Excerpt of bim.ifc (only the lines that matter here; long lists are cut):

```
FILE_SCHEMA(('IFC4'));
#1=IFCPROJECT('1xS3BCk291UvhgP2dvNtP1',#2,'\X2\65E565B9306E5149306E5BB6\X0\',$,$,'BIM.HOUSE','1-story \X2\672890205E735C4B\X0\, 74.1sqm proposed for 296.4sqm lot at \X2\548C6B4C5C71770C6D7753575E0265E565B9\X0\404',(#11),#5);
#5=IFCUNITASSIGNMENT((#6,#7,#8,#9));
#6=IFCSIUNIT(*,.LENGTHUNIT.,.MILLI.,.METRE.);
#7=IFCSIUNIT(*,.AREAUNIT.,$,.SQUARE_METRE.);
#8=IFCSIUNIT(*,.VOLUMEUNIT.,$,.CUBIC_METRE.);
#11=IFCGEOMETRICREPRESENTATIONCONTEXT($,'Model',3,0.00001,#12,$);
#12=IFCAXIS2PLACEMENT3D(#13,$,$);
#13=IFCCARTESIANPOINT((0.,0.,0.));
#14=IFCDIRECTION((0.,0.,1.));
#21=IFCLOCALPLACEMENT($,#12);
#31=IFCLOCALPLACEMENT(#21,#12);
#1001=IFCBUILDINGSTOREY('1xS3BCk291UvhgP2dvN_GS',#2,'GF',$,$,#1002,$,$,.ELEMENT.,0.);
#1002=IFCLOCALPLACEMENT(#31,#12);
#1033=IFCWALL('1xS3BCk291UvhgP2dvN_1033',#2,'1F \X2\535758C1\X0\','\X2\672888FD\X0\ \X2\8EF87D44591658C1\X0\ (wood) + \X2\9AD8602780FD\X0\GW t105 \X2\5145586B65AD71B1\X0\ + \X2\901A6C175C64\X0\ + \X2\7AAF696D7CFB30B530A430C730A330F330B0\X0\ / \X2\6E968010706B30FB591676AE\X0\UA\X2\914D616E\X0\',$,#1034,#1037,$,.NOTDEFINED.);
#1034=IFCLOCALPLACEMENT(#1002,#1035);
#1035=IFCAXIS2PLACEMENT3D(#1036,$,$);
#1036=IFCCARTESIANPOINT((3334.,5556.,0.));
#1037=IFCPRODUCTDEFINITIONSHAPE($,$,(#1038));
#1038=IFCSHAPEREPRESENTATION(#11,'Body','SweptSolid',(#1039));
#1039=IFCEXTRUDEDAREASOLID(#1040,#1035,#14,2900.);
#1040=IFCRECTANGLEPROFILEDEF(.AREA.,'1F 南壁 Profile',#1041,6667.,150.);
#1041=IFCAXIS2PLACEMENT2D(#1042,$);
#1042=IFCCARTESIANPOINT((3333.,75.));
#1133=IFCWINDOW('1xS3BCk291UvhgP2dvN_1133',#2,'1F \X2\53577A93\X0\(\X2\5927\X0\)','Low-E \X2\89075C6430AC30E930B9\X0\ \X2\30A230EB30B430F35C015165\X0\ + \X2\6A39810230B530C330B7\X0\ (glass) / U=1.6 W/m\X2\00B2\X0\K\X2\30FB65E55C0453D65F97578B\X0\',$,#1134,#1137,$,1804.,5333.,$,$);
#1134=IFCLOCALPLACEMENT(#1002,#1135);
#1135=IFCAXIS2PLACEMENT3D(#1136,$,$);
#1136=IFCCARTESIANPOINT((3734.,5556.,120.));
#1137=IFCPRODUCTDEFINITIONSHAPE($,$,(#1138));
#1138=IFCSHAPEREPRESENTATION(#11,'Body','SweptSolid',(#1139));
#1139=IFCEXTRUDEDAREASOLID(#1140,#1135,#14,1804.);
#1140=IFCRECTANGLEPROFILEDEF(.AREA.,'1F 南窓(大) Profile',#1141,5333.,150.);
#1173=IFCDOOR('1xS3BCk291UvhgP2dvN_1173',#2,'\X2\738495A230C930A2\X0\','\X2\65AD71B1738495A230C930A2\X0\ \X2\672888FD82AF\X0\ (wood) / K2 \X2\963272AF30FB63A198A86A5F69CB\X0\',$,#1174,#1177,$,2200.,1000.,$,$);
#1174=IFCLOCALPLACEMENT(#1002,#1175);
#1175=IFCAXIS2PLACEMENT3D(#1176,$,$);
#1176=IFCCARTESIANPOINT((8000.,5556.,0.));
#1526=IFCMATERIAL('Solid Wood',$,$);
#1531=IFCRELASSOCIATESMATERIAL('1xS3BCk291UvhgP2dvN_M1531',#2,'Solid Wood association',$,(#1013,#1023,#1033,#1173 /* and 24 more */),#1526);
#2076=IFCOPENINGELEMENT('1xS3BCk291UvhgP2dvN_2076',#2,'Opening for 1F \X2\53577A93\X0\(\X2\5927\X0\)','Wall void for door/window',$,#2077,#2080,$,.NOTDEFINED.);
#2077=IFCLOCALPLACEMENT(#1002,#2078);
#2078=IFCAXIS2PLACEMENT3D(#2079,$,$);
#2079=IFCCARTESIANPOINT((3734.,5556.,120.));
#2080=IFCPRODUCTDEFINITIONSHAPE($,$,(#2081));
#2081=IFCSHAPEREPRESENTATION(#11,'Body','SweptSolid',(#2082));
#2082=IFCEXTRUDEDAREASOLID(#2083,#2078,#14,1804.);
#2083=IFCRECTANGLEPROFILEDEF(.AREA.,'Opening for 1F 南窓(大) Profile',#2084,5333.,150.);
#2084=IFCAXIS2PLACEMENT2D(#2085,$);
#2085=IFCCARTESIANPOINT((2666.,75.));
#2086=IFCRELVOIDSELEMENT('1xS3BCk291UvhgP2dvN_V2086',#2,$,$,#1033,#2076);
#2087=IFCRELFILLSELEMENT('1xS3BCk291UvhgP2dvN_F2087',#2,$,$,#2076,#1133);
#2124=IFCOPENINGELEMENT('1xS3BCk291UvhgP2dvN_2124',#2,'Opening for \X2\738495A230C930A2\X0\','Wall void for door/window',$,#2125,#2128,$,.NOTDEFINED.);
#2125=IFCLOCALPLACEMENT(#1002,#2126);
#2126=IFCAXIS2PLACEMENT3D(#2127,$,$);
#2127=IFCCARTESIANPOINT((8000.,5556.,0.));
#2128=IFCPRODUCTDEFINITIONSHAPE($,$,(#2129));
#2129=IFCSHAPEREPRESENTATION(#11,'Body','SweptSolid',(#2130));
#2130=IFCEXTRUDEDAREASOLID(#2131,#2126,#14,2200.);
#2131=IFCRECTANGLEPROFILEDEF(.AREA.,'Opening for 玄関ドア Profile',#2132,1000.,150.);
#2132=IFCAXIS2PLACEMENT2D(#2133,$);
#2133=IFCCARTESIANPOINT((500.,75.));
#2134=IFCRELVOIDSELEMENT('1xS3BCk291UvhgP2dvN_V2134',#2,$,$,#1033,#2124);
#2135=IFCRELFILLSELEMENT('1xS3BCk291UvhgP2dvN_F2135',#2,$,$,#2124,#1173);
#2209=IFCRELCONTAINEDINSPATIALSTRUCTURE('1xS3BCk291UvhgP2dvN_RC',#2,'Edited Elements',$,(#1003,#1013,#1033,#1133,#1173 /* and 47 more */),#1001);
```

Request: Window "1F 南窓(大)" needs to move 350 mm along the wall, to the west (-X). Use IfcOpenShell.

```python
import ifcopenshell
import ifcopenshell.api.geometry
import ifcopenshell.util.placement

model = ifcopenshell.open("bim.ifc")

window = model.by_guid("1xS3BCk291UvhgP2dvN_1133")
opening = window.FillsVoids[0].RelatingOpeningElement
wall = opening.VoidsElements[0].RelatingBuildingElement

wall_matrix = ifcopenshell.util.placement.get_local_placement(wall.ObjectPlacement)
shift = wall_matrix[:3, 0] * -350.0
before = ifcopenshell.util.placement.get_local_placement(window.ObjectPlacement)[:3, 3].copy()

# The window is not placed relative to its opening, so move both.
for product in (opening, window):
    matrix = ifcopenshell.util.placement.get_local_placement(product.ObjectPlacement)
    matrix[:3, 3] += shift
    ifcopenshell.api.geometry.edit_object_placement(model, product=product, matrix=matrix, is_si=False)

after = ifcopenshell.util.placement.get_local_placement(window.ObjectPlacement)[:3, 3]
print("window moved by", (after - before).round(3) + 0.0)

model.write("bim-out.ifc")
```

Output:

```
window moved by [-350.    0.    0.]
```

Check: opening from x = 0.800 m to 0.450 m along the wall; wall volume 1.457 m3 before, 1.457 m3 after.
